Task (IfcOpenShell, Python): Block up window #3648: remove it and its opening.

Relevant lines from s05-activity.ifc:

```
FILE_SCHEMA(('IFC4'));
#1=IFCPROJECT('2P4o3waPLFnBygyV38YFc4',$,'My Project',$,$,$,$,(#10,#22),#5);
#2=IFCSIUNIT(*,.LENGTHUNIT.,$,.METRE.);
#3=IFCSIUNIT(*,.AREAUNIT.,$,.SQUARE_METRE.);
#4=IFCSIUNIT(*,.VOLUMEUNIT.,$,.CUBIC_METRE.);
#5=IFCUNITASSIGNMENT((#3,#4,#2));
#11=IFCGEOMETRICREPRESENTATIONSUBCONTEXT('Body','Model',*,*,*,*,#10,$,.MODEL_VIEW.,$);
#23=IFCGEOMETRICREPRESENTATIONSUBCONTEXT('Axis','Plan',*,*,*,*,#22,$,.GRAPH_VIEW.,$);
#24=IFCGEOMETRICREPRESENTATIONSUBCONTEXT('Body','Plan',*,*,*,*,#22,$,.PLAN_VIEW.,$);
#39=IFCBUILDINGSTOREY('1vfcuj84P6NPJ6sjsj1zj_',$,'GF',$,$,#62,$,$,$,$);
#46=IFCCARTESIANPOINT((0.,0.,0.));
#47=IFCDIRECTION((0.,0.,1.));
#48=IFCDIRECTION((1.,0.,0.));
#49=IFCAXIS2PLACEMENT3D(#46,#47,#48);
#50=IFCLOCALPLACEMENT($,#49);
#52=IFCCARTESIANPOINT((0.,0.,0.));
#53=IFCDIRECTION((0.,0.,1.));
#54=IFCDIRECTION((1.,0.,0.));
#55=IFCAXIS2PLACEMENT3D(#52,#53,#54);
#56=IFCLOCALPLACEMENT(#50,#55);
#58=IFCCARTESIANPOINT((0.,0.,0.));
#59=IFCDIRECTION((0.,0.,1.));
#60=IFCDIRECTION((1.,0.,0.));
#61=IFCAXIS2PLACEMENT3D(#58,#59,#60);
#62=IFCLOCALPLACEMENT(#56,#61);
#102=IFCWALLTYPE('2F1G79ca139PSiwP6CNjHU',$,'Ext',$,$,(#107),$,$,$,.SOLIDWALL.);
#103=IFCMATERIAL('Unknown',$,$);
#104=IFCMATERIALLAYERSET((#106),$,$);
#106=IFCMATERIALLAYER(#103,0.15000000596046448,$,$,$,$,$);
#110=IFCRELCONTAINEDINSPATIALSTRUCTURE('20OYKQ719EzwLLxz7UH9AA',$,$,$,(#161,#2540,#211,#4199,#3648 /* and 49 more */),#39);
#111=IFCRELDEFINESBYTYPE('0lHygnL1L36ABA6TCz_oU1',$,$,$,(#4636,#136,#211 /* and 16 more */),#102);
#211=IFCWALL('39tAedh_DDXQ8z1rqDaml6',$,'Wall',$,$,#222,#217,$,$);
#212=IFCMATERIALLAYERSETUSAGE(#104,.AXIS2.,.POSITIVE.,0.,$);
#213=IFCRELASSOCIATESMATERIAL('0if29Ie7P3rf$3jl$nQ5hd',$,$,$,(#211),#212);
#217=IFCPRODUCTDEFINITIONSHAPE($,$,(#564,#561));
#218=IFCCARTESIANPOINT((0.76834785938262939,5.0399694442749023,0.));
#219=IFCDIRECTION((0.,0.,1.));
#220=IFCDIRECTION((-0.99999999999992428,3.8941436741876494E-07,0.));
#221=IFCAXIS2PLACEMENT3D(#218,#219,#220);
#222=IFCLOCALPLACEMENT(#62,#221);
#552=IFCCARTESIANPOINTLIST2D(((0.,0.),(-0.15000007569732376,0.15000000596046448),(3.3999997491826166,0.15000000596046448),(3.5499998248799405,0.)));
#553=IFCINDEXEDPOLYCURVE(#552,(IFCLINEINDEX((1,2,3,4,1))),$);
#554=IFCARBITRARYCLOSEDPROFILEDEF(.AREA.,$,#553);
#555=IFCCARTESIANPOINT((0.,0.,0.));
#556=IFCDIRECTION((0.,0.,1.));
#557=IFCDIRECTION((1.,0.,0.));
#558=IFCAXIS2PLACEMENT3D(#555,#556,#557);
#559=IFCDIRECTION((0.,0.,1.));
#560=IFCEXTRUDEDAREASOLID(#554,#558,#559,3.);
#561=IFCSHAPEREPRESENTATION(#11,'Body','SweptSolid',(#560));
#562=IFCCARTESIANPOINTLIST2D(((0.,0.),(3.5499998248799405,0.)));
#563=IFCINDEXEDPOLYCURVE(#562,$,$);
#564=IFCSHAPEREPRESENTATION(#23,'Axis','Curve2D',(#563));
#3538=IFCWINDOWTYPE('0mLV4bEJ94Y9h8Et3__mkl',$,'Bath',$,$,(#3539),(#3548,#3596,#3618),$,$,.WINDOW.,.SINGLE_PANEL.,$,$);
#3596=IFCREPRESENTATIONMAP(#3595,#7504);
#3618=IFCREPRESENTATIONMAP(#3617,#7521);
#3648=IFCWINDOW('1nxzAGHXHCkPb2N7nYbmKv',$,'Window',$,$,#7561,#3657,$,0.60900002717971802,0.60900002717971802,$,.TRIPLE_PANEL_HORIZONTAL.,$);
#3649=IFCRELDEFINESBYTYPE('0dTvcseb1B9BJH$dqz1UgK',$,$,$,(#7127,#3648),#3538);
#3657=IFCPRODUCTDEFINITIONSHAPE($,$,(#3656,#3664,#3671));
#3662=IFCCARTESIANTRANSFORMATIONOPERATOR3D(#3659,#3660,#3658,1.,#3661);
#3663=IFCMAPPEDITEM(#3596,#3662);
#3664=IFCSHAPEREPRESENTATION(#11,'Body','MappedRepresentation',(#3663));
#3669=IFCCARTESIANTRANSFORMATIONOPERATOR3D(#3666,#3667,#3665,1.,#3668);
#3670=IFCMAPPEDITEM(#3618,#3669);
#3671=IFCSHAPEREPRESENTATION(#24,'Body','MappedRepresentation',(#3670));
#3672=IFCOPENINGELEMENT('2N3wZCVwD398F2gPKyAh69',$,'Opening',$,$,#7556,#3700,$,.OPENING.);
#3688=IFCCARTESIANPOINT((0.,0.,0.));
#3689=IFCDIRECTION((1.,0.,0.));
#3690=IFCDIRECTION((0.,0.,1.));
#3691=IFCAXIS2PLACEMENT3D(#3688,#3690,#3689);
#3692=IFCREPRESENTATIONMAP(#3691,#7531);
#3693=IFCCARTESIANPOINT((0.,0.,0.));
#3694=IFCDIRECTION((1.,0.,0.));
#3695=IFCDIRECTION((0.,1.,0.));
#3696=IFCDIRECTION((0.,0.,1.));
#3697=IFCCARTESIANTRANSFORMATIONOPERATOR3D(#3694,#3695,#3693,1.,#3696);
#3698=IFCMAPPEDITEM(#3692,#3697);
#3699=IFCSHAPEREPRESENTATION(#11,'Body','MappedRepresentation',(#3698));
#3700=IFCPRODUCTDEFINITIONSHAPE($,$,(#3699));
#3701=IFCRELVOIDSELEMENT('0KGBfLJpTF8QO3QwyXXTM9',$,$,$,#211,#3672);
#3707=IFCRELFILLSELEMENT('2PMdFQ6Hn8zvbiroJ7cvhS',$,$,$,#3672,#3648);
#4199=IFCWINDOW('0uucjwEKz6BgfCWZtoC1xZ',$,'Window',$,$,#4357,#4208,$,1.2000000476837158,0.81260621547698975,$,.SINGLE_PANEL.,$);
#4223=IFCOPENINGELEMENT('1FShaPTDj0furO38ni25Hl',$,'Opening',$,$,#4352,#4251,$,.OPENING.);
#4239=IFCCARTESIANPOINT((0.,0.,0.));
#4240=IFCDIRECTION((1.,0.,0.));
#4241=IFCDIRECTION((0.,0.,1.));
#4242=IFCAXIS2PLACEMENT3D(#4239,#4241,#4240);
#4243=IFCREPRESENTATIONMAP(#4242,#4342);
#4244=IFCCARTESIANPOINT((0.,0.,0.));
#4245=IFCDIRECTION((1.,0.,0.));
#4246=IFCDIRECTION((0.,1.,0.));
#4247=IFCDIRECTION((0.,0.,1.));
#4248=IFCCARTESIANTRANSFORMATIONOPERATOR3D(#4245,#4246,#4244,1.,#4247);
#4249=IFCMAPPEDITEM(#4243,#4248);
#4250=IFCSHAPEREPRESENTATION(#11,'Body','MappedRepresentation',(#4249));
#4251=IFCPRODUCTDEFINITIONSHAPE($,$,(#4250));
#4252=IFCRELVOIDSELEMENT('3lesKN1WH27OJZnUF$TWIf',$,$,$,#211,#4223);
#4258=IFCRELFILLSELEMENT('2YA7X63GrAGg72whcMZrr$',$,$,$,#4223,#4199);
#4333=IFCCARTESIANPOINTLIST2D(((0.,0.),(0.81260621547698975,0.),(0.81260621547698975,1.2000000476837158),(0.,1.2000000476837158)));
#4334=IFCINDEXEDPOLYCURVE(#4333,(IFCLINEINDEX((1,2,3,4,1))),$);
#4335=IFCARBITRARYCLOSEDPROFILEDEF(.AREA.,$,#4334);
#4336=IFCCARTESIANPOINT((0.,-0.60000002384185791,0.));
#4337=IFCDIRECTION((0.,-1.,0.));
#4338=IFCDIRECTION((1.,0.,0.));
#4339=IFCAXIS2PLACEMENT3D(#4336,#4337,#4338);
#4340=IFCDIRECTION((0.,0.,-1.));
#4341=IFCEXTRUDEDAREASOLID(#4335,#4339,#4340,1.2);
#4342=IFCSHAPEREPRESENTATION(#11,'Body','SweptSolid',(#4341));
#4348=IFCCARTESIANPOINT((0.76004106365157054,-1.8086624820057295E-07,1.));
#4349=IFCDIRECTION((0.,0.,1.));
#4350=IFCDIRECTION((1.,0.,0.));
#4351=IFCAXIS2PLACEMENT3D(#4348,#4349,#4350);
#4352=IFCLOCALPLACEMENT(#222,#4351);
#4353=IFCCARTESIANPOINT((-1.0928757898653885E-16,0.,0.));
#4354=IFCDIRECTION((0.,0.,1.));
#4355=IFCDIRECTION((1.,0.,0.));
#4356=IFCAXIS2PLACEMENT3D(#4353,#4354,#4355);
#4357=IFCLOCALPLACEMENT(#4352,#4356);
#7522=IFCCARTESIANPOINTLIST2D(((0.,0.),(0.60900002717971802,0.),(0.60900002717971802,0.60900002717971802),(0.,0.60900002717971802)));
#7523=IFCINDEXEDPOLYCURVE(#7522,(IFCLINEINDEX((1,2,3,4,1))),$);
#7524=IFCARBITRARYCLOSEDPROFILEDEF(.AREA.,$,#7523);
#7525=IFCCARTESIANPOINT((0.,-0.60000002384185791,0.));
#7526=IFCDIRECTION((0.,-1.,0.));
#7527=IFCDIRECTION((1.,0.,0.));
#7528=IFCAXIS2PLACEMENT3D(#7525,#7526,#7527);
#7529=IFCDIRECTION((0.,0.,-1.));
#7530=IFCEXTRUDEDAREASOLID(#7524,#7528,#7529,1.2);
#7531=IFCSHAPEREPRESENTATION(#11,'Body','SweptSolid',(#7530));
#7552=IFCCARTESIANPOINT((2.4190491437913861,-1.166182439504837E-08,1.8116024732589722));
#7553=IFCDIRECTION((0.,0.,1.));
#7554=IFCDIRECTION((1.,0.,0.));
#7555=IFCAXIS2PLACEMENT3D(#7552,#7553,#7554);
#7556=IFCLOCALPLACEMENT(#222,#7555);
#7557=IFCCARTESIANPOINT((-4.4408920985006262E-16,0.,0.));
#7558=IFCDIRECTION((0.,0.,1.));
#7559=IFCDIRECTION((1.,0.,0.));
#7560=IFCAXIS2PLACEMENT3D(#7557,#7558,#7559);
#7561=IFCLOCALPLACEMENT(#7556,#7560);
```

```python
import ifcopenshell
import ifcopenshell.api.feature
import ifcopenshell.api.root
import ifcopenshell.geom
import ifcopenshell.util.shape

model = ifcopenshell.open("s05-activity.ifc")
settings = ifcopenshell.geom.settings()


def volume(element):
    """Net volume in cubic metres, openings subtracted."""
    shape = ifcopenshell.geom.create_shape(settings, element)
    return ifcopenshell.util.shape.get_volume(shape.geometry)


window = model.by_guid("1nxzAGHXHCkPb2N7nYbmKv")
opening = window.FillsVoids[0].RelatingOpeningElement
wall = opening.VoidsElements[0].RelatingBuildingElement
before = volume(wall)

ifcopenshell.api.root.remove_product(model, product=window)
ifcopenshell.api.feature.remove_feature(model, feature=opening)

after = volume(wall)

print(f"wall volume {before:.3f} -> {after:.3f} m3")

model.write("s05-activity_updated.ifc")
```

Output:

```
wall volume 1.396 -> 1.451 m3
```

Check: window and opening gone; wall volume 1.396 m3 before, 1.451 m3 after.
